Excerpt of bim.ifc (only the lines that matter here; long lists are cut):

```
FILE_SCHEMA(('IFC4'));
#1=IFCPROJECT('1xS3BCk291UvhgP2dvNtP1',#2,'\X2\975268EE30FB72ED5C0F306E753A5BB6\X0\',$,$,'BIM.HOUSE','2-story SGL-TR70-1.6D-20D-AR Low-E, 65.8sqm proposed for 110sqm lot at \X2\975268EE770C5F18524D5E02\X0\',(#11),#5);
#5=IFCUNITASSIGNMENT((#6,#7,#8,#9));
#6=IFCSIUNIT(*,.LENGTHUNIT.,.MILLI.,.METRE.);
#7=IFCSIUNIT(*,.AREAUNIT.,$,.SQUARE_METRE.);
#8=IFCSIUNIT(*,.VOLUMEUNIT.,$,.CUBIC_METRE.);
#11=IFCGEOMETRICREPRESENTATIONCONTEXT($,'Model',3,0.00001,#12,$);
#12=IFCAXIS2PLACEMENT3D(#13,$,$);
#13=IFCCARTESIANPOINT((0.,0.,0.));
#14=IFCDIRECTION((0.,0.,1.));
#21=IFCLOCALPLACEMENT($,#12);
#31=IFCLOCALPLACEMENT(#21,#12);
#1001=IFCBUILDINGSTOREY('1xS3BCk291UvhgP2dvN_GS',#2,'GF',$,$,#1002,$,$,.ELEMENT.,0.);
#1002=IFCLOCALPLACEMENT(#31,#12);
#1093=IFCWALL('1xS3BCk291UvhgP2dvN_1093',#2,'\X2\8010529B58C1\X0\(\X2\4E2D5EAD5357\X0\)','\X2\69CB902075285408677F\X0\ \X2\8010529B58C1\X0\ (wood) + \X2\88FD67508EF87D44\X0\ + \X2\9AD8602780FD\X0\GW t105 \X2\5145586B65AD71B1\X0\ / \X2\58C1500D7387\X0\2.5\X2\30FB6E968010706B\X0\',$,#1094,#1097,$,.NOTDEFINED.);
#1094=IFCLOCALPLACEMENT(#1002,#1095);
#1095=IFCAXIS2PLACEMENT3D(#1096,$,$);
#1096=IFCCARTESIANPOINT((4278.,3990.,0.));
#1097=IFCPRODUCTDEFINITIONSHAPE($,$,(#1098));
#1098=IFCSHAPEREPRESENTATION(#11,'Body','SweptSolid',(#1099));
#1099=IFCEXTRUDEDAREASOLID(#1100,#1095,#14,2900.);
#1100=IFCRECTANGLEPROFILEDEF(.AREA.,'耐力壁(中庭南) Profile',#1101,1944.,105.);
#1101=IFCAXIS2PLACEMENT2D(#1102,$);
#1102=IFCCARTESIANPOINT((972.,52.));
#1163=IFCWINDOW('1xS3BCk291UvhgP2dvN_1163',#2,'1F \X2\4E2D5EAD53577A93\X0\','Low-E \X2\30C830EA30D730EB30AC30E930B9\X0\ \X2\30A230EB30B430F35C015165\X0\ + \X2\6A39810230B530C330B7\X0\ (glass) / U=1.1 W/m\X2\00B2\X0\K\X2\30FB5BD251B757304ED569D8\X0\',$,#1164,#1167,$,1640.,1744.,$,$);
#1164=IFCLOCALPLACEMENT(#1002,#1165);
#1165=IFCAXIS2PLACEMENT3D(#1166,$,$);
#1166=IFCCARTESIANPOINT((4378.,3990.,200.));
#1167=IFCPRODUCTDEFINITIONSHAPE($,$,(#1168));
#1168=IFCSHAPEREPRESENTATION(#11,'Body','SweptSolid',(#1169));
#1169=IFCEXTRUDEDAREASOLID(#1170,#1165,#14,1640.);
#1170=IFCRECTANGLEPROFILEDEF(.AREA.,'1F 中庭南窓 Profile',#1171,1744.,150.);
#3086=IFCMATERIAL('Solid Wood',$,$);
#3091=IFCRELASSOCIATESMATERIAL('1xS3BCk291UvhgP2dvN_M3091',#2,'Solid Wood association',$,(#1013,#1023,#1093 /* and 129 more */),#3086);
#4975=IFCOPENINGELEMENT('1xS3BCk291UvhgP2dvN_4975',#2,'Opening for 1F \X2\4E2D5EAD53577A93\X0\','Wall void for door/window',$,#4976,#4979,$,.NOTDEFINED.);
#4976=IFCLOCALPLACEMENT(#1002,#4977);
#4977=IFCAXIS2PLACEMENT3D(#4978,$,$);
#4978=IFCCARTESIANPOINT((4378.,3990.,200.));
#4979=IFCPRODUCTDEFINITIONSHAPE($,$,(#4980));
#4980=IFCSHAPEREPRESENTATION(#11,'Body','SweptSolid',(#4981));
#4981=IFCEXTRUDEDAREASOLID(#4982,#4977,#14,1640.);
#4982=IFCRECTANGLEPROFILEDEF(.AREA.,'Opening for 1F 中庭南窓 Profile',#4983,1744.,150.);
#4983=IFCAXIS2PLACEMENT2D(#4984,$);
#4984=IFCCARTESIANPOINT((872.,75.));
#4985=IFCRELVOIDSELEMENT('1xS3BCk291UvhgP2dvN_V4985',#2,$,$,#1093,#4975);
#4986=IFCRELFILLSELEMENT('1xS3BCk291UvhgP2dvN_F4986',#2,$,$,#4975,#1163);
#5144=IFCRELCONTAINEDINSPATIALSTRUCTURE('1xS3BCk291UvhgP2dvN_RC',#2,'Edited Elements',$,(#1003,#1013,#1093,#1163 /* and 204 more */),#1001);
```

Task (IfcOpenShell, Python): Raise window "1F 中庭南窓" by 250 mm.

```python
import numpy as np
import ifcopenshell
import ifcopenshell.api.geometry
import ifcopenshell.util.placement
import ifcopenshell.util.unit

model = ifcopenshell.open("bim.ifc")
unit_scale = ifcopenshell.util.unit.calculate_unit_scale(model)

window = model.by_guid("1xS3BCk291UvhgP2dvN_1163")
opening = window.FillsVoids[0].RelatingOpeningElement
dz = 0.25 / unit_scale

shift = np.array([0.0, 0.0, dz])
# The window is not placed relative to its opening, so move both.
for product in (opening, window):
    matrix = ifcopenshell.util.placement.get_local_placement(product.ObjectPlacement)
    matrix[:3, 3] += shift
    ifcopenshell.api.geometry.edit_object_placement(model, product=product, matrix=matrix, is_si=False)

print(f"moved by {dz * unit_scale:+.3f} m")

model.write("bim-out.ifc")
```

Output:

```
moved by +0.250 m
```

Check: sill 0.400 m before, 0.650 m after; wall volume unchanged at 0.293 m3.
